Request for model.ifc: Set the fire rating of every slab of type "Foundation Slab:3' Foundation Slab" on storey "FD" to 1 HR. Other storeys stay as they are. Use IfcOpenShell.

First a look at what the model holds.

```python
import ifcopenshell
import ifcopenshell.util.element

model = ifcopenshell.open("model.ifc")
print(model.schema)
storey = next(s for s in model.by_type("IfcBuildingStorey") if s.Name == "FD")
slabs = [e for e in ifcopenshell.util.element.get_decomposition(storey) if e.is_a("IfcSlab")]
seen = {}
for e in slabs:
    element_type = ifcopenshell.util.element.get_type(e)
    key = (element_type.Name if element_type != e and element_type else None, ifcopenshell.util.element.get_pset(e, "Pset_SlabCommon", "FireRating"))
    seen[key] = seen.get(key, 0) + 1
for (name, value), count in sorted(seen.items(), key=str):
    print(count, "x", name, "|", value)
```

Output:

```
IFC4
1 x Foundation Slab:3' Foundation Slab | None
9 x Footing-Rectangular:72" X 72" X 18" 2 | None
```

```python
import ifcopenshell
import ifcopenshell.api.pset
import ifcopenshell.util.element

model = ifcopenshell.open("model.ifc")

storey = next(s for s in model.by_type("IfcBuildingStorey") if s.Name == "FD")
slabs = [e for e in ifcopenshell.util.element.get_decomposition(storey) if e.is_a("IfcSlab")]

count = 0
for e in slabs:
    element_type = ifcopenshell.util.element.get_type(e)
    if element_type in (None, e) or element_type.Name != "Foundation Slab:3' Foundation Slab":
        continue
    # add_pset returns the element's existing set when there is one.
    pset = ifcopenshell.api.pset.add_pset(model, product=e, name="Pset_SlabCommon")
    ifcopenshell.api.pset.edit_pset(model, pset=pset, properties={"FireRating": "1 HR"})
    count += 1

print(count, "slabs updated")

model.write("model_rev.ifc")
```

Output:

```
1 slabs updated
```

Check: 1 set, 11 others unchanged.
